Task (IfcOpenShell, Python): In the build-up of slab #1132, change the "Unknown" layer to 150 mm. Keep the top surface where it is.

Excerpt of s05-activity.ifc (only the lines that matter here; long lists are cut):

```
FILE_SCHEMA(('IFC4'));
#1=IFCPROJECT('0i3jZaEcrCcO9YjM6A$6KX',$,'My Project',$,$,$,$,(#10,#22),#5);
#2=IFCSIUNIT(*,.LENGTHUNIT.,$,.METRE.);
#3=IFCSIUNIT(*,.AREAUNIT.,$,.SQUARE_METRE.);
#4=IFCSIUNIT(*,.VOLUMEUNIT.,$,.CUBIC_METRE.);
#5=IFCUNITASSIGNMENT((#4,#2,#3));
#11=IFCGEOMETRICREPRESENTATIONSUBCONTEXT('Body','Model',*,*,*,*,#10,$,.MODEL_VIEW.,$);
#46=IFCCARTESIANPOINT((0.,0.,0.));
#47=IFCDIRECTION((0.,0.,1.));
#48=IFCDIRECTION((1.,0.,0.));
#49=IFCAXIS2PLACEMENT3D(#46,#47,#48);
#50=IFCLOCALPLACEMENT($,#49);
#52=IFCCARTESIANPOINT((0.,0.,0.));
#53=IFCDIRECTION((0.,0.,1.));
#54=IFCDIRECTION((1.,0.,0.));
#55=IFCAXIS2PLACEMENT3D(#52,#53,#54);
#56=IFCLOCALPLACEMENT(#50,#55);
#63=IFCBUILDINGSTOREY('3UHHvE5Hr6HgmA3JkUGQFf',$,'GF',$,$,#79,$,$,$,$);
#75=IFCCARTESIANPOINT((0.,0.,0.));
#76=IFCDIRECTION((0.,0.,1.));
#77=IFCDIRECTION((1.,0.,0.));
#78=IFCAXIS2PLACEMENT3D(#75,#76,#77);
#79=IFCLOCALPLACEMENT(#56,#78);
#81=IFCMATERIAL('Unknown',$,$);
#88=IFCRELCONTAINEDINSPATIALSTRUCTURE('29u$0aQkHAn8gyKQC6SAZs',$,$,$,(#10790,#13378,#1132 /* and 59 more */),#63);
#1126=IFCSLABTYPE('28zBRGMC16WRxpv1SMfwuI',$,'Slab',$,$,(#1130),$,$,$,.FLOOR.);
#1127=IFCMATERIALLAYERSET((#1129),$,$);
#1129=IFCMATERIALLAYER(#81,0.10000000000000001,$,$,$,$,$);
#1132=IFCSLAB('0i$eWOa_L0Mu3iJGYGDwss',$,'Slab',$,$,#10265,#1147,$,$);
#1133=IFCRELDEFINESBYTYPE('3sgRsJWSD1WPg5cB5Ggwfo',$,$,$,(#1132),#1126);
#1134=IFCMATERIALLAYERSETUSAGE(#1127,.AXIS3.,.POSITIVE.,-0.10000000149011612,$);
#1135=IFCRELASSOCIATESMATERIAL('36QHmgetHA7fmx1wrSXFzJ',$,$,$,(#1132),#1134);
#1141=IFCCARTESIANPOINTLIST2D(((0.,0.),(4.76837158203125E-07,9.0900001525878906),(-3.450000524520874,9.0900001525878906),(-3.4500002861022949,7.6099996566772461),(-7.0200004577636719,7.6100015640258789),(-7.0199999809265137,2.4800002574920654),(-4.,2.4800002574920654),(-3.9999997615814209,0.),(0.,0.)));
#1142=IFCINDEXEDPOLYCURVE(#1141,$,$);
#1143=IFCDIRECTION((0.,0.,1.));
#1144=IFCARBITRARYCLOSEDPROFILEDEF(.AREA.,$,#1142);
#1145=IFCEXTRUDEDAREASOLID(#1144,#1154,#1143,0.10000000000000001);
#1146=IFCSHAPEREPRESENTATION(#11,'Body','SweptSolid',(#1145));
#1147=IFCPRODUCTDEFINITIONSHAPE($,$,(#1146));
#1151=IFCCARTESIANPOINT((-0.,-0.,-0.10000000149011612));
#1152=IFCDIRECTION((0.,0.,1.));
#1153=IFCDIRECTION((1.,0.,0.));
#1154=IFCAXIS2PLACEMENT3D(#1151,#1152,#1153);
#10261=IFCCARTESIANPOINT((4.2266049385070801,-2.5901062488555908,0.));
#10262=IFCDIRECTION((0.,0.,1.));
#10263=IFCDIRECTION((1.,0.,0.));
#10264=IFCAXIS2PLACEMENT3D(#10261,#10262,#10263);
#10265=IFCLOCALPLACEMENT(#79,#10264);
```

```python
import ifcopenshell
import ifcopenshell.util.element
import ifcopenshell.util.representation

model = ifcopenshell.open("s05-activity.ifc")

layer_set = model.by_id(1127)
layer = next(l for l in layer_set.MaterialLayers if l.Material and l.Material.Name == "Unknown")
change = 0.15 - layer.LayerThickness
layer.LayerThickness += change

# Geometry does not follow the layer set by itself.
slabs = [e for e in ifcopenshell.util.element.get_elements_by_material(model, layer_set) if e.is_a("IfcSlab")]
for slab in sorted(slabs, key=lambda e: e.id()):
    body = ifcopenshell.util.representation.get_representation(slab, "Model", "Body")
    solid = body.Items[0]
    old_depth = solid.Depth
    solid.Depth += change
    # Extruded upwards: lower the start of the extrusion so the top stays.
    x, y, z = solid.Position.Location.Coordinates
    solid.Position.Location = model.createIfcCartesianPoint((x, y, z - change))
    print(slab.id(), f"{old_depth:g} -> {solid.Depth:g}")

# The layers are counted up from the underside, which has moved.
for usage in {ifcopenshell.util.element.get_material(slab) for slab in slabs}:
    usage.OffsetFromReferenceLine -= change

model.write("s05-activity_edited.ifc")
```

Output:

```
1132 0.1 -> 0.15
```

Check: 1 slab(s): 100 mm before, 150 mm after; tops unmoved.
